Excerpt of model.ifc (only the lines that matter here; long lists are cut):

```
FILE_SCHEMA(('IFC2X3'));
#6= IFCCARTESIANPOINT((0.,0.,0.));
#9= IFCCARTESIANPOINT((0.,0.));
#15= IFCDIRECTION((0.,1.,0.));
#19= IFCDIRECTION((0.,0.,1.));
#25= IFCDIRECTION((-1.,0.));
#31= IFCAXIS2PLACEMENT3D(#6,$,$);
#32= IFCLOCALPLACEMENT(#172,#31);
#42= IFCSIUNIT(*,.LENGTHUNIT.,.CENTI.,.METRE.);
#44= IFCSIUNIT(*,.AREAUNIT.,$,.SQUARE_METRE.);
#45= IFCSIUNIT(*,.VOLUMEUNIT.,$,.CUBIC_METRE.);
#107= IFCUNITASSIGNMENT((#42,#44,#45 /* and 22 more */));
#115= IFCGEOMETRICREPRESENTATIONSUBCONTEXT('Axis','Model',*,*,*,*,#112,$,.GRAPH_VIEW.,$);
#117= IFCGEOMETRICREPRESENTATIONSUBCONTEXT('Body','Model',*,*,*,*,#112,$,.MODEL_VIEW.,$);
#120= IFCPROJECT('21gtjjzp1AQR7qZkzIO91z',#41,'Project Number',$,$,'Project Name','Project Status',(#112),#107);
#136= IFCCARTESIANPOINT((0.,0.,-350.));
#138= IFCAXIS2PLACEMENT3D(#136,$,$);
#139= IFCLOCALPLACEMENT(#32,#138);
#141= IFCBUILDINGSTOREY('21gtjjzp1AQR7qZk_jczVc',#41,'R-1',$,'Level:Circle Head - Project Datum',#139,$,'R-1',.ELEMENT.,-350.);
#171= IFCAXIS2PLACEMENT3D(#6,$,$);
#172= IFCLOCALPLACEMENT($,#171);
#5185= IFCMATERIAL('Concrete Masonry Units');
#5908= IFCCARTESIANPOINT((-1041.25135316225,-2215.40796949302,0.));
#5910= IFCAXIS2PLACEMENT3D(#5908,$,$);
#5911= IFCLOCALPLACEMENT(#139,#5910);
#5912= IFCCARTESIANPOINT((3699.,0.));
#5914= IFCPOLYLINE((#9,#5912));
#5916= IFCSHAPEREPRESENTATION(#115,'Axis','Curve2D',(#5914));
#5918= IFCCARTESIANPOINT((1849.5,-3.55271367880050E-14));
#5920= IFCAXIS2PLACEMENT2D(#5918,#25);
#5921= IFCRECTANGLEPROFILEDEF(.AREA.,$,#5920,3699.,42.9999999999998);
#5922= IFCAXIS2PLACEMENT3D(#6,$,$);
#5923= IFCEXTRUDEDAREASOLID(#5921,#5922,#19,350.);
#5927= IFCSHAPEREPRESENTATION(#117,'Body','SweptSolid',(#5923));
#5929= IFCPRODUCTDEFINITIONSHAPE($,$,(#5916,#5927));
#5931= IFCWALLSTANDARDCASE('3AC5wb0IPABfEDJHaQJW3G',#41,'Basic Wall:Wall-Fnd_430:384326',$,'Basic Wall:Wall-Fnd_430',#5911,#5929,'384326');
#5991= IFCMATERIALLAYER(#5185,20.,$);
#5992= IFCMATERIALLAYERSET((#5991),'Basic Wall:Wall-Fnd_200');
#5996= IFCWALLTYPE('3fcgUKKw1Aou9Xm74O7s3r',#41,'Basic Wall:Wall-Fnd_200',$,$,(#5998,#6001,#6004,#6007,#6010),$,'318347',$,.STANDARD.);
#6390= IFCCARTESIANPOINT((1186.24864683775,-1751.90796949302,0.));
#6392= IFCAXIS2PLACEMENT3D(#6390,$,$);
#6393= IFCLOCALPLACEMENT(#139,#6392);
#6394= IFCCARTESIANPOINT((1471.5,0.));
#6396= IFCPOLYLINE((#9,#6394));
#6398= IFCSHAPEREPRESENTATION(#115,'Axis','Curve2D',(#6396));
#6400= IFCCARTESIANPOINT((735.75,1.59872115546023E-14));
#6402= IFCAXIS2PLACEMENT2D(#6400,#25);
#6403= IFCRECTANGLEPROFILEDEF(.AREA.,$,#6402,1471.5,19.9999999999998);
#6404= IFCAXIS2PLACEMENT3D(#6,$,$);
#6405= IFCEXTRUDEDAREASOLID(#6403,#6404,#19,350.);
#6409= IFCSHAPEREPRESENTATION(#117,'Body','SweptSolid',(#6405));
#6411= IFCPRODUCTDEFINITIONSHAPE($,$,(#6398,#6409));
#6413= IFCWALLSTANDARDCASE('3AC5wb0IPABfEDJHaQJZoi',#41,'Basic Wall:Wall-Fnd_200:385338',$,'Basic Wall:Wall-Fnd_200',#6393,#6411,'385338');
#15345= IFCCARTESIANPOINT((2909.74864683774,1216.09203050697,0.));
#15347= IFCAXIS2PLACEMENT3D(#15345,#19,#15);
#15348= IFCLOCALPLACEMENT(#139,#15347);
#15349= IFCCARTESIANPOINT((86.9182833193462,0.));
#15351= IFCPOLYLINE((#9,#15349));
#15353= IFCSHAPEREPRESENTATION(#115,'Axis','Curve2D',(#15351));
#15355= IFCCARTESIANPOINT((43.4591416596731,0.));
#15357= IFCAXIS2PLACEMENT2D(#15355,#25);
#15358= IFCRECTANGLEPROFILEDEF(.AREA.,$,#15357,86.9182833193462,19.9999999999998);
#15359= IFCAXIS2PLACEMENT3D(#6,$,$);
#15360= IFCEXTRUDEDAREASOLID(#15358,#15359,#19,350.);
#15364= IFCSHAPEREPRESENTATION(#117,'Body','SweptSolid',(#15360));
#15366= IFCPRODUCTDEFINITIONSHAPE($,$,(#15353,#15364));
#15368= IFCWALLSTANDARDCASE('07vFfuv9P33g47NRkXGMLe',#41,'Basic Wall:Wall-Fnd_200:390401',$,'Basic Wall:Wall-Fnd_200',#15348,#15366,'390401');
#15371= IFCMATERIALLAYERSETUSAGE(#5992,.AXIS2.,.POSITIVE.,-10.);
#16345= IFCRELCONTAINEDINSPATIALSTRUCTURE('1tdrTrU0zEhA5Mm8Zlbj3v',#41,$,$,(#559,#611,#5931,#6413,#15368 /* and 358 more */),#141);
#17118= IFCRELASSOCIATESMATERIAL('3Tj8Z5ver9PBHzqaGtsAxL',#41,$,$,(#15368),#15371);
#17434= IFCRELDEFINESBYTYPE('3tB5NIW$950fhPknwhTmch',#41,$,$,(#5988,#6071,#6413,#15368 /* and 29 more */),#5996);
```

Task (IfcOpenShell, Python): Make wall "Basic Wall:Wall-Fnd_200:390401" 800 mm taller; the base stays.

```python
import ifcopenshell
import ifcopenshell.geom
import ifcopenshell.util.representation
import ifcopenshell.util.shape
import ifcopenshell.util.unit

model = ifcopenshell.open("model.ifc")
unit_scale = ifcopenshell.util.unit.calculate_unit_scale(model)
settings = ifcopenshell.geom.settings()


def volume(element):
    """Net volume in cubic metres, openings subtracted."""
    shape = ifcopenshell.geom.create_shape(settings, element)
    return ifcopenshell.util.shape.get_volume(shape.geometry)


wall = model.by_guid("07vFfuv9P33g47NRkXGMLe")
before = volume(wall)

body = ifcopenshell.util.representation.get_representation(wall, "Model", "Body")
solid = body.Items[0]
old_height = solid.Depth
solid.Depth += 0.8 / unit_scale
after = volume(wall)

print(f"height {old_height:g} -> {solid.Depth:g}, volume {before:.3f} -> {after:.3f} m3")

model.write("model_edited.ifc")
```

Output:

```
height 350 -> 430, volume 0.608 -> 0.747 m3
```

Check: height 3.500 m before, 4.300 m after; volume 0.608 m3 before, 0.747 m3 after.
